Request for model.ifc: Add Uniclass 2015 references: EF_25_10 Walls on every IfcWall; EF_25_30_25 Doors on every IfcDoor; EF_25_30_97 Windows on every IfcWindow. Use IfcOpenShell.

First a look at what the model holds.

```python
import ifcopenshell

model = ifcopenshell.open("model.ifc")
print(model.schema)
print("classifications:", [c.Name for c in model.by_type("IfcClassification")])
for ifc_class in ("IfcDoor", "IfcRoof", "IfcStair", "IfcWall", "IfcWindow"):
    print(ifc_class, len(model.by_type(ifc_class)))
```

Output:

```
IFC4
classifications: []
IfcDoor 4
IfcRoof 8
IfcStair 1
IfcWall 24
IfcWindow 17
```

```python
import ifcopenshell
import ifcopenshell.api.classification

model = ifcopenshell.open("model.ifc")

system = ifcopenshell.api.classification.add_classification(model, classification="Uniclass 2015")

codes = {
    "IfcWall": ("EF_25_10", "Walls"),
    "IfcDoor": ("EF_25_30_25", "Doors"),
    "IfcWindow": ("EF_25_30_97", "Windows"),
}
for ifc_class, (code, name) in codes.items():
    products = model.by_type(ifc_class)
    ifcopenshell.api.classification.add_reference(
        model, products=products, classification=system, identification=code, name=name
    )
    print(code, len(products))

model.write("model_v2.ifc")
```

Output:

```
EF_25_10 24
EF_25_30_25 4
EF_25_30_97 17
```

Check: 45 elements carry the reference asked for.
